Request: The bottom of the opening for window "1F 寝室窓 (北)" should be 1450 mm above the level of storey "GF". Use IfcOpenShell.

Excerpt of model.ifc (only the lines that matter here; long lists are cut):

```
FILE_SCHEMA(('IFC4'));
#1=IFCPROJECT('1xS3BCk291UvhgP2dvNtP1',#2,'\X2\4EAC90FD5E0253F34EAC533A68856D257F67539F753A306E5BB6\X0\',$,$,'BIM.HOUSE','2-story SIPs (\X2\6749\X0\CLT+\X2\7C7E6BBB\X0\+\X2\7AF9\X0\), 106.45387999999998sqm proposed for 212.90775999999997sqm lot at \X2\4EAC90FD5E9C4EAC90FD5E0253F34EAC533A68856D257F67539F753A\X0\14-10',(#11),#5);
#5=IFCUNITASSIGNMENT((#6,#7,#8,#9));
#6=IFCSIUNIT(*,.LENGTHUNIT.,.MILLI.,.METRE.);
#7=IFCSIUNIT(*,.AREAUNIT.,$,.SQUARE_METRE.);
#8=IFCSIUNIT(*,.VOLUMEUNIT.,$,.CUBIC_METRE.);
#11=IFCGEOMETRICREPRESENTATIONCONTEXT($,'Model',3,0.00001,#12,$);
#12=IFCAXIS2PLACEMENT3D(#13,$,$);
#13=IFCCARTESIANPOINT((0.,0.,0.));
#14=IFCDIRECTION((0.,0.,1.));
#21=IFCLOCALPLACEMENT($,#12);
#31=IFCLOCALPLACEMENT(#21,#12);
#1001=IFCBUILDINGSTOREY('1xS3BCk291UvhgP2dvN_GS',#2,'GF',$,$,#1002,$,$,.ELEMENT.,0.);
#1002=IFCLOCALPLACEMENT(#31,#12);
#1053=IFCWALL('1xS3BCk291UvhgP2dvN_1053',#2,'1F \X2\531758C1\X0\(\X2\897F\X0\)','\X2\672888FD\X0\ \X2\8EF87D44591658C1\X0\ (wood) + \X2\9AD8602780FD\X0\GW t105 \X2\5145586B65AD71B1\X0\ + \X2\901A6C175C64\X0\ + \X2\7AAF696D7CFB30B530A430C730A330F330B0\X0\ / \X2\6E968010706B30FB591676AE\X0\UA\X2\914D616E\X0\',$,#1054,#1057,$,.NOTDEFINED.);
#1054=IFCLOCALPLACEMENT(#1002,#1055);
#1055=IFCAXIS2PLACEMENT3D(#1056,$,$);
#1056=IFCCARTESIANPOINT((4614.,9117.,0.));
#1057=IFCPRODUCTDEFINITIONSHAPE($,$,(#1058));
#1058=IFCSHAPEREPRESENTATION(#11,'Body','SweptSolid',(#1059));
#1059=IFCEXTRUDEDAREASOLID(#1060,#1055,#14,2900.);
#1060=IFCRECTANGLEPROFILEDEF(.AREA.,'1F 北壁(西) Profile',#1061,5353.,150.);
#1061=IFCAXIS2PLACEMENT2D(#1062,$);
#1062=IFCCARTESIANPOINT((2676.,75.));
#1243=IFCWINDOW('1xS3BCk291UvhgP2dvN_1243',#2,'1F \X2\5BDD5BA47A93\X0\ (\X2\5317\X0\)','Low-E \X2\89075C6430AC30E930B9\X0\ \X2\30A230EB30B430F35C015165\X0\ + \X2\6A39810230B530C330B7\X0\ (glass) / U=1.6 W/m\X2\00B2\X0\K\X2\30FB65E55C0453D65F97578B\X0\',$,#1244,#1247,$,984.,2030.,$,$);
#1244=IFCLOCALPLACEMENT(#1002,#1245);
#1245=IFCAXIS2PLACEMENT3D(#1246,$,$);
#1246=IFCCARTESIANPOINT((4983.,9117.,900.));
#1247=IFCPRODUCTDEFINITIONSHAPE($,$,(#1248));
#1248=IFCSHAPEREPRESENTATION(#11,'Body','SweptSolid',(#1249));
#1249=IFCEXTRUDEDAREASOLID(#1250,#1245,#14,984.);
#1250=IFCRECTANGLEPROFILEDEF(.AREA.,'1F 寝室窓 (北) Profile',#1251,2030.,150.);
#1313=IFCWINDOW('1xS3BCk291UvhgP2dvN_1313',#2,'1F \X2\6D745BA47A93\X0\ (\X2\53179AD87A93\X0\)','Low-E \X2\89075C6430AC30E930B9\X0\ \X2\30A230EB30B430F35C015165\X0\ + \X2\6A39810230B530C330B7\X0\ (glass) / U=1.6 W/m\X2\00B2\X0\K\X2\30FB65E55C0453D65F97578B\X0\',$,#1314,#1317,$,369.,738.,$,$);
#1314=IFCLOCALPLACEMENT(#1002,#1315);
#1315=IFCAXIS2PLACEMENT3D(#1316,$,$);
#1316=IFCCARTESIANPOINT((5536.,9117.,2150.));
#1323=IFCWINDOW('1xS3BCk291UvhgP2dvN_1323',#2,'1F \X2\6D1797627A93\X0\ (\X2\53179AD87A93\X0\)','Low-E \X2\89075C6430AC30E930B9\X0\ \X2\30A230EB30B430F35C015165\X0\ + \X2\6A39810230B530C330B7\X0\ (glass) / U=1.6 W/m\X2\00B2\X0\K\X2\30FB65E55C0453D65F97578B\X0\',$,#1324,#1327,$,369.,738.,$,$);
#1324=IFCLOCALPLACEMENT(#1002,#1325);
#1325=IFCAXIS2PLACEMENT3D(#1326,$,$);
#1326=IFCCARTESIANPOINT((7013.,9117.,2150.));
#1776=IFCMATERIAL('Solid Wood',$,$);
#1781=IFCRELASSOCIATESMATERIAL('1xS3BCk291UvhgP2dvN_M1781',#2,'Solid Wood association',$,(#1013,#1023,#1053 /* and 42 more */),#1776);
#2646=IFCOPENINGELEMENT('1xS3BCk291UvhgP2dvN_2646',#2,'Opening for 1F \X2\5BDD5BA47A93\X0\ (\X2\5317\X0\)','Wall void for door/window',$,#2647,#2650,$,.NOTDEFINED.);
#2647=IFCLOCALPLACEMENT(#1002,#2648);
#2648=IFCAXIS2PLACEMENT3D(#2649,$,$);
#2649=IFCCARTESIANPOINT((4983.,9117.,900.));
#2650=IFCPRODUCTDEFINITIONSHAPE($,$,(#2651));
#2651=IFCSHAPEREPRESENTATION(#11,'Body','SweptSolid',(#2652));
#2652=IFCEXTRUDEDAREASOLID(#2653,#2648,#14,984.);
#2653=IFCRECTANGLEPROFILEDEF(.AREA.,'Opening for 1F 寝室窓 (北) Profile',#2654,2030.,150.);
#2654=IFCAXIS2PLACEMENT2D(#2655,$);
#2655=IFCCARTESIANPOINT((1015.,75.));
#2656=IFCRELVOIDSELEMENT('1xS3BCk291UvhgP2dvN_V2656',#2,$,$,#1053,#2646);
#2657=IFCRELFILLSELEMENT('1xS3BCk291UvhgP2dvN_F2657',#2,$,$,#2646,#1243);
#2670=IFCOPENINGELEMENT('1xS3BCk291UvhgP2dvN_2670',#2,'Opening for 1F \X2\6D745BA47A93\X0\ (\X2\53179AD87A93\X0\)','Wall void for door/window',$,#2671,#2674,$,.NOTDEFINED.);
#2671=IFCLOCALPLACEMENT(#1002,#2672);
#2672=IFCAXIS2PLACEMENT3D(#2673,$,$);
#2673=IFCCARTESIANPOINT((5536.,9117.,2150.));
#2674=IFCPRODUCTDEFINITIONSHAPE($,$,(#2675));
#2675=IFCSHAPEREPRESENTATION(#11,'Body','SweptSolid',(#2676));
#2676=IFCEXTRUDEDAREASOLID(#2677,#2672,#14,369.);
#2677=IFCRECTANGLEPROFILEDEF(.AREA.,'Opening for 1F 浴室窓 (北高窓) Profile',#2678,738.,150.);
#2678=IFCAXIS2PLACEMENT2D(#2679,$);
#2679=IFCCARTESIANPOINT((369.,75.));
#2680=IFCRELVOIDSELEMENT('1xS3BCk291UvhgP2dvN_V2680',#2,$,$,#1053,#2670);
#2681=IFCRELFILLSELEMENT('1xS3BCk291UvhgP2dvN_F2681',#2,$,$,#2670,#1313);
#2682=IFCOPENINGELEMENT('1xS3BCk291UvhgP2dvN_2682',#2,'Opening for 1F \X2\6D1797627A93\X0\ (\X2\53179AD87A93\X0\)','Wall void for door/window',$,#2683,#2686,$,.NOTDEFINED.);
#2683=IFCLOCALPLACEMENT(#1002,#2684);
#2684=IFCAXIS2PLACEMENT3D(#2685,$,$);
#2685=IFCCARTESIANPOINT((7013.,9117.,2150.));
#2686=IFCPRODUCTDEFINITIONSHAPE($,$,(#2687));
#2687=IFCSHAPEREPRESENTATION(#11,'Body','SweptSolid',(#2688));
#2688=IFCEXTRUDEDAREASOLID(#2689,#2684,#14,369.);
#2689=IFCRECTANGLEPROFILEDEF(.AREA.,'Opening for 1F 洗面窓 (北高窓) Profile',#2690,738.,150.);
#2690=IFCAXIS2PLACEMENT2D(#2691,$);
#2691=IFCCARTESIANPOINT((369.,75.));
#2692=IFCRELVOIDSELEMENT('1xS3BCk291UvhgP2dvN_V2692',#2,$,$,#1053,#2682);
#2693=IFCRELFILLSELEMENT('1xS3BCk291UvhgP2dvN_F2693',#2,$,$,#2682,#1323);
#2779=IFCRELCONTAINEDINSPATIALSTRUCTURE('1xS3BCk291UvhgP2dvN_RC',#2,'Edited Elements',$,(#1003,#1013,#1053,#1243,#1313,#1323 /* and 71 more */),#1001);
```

```python
import numpy as np
import ifcopenshell
import ifcopenshell.api.geometry
import ifcopenshell.geom
import ifcopenshell.util.element
import ifcopenshell.util.placement
import ifcopenshell.util.shape
import ifcopenshell.util.unit

model = ifcopenshell.open("model.ifc")
unit_scale = ifcopenshell.util.unit.calculate_unit_scale(model)

window = model.by_guid("1xS3BCk291UvhgP2dvN_1243")
opening = window.FillsVoids[0].RelatingOpeningElement
storey = ifcopenshell.util.element.get_container(window, ifc_class="IfcBuildingStorey")
level = ifcopenshell.util.placement.get_local_placement(storey.ObjectPlacement)[2, 3]

# The opening's origin need not be at the sill, so measure its lowest point.
shape = ifcopenshell.geom.create_shape(ifcopenshell.geom.settings(), opening)
bottom = ifcopenshell.util.shape.get_shape_bottom_elevation(shape, shape.geometry) / unit_scale
dz = level + 1450.0 - bottom

shift = np.array([0.0, 0.0, dz])
# The window is not placed relative to its opening, so move both.
for product in (opening, window):
    matrix = ifcopenshell.util.placement.get_local_placement(product.ObjectPlacement)
    matrix[:3, 3] += shift
    ifcopenshell.api.geometry.edit_object_placement(model, product=product, matrix=matrix, is_si=False)

print(f"moved by {dz * unit_scale:+.3f} m")

model.write("model_edited.ifc")
```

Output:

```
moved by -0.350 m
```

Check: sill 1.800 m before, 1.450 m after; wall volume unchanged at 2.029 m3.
